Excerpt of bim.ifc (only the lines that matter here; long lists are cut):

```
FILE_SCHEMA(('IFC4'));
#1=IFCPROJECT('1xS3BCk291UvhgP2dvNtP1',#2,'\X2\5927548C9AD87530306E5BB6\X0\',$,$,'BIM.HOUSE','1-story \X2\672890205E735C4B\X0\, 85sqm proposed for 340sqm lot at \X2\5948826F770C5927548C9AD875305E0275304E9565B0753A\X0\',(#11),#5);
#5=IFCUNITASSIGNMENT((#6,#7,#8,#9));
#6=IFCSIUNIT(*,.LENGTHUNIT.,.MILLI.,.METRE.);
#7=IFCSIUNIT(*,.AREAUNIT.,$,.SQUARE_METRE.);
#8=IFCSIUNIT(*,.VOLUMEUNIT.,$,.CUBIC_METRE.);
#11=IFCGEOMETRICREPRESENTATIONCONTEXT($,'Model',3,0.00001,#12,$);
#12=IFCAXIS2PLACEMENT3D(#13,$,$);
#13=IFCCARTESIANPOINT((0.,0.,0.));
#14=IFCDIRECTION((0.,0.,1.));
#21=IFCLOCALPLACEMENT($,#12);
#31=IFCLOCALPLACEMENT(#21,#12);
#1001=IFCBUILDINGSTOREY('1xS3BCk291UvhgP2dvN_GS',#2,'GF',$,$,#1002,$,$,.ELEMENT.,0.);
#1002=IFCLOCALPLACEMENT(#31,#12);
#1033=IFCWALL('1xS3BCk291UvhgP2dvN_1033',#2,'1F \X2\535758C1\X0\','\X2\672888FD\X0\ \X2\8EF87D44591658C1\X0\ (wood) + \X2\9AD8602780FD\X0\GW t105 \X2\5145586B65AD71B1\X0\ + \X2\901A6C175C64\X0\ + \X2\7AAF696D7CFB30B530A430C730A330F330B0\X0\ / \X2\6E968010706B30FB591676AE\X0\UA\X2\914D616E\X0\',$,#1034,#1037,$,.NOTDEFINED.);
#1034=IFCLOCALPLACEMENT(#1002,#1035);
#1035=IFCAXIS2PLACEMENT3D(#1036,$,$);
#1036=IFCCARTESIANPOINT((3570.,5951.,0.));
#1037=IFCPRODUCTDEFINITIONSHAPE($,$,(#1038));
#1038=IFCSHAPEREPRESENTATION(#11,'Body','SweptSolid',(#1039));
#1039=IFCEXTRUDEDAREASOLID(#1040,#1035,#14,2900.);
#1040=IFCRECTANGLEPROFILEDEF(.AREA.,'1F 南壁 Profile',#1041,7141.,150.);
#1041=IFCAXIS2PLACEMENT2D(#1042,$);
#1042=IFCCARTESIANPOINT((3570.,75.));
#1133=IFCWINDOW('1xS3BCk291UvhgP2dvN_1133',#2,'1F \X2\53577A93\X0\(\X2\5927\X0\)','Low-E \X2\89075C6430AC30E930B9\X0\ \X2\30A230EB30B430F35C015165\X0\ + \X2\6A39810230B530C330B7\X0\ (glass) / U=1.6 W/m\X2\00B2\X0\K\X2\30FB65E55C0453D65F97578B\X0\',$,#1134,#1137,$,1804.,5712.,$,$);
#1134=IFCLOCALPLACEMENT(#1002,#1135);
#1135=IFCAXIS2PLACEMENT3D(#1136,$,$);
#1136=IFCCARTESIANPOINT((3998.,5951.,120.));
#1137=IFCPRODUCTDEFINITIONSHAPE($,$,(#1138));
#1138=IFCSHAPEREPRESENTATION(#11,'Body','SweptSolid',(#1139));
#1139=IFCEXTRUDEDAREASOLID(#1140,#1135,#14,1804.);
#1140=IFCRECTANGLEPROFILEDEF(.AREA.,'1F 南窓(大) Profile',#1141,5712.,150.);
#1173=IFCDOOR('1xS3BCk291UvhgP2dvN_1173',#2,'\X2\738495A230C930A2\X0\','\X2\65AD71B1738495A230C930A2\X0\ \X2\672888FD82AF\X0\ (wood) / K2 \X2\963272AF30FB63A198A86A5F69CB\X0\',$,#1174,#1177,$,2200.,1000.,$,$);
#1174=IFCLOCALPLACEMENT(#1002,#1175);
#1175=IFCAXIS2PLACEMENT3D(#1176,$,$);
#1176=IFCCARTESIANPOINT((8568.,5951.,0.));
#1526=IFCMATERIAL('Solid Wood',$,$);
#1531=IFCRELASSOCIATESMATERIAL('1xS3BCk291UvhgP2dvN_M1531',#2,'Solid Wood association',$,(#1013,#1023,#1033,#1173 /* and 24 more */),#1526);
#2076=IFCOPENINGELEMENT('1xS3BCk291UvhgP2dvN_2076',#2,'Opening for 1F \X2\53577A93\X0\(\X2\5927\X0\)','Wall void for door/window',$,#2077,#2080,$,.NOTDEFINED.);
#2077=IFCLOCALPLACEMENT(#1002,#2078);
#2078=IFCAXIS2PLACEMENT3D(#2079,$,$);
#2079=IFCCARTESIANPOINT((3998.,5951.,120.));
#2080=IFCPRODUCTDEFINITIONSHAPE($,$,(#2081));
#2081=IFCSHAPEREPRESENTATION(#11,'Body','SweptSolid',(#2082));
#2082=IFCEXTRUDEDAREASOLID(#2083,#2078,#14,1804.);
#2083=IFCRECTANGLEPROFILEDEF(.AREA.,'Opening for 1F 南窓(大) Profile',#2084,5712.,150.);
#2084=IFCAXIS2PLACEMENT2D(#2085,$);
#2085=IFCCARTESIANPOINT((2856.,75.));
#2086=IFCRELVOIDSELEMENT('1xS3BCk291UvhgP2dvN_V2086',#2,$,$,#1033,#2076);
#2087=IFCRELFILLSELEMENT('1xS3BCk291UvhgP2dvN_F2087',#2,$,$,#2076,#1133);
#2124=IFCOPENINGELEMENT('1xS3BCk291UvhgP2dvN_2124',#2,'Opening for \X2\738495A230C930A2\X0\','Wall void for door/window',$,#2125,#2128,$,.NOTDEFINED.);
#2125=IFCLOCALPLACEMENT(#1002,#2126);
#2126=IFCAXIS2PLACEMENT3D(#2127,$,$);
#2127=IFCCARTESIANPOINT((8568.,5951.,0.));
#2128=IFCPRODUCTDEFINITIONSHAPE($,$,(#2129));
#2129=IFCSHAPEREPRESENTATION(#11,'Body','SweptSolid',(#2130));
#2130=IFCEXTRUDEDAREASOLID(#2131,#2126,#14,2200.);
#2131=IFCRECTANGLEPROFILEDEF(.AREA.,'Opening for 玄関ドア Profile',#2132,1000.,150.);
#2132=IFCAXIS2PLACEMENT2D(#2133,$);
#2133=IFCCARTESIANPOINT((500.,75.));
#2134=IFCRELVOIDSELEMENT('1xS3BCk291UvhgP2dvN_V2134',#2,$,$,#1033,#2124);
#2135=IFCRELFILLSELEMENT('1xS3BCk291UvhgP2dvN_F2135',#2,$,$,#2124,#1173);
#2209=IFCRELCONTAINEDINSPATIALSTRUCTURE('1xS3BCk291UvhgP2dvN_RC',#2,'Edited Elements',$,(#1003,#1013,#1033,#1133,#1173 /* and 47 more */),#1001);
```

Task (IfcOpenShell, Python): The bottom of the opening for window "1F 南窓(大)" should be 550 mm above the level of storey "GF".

```python
import numpy as np
import ifcopenshell
import ifcopenshell.api.geometry
import ifcopenshell.geom
import ifcopenshell.util.element
import ifcopenshell.util.placement
import ifcopenshell.util.shape
import ifcopenshell.util.unit

model = ifcopenshell.open("bim.ifc")
unit_scale = ifcopenshell.util.unit.calculate_unit_scale(model)

window = model.by_guid("1xS3BCk291UvhgP2dvN_1133")
opening = window.FillsVoids[0].RelatingOpeningElement
storey = ifcopenshell.util.element.get_container(window, ifc_class="IfcBuildingStorey")
level = ifcopenshell.util.placement.get_local_placement(storey.ObjectPlacement)[2, 3]

# The opening's origin need not be at the sill, so measure its lowest point.
shape = ifcopenshell.geom.create_shape(ifcopenshell.geom.settings(), opening)
bottom = ifcopenshell.util.shape.get_shape_bottom_elevation(shape, shape.geometry) / unit_scale
dz = level + 0.55 / unit_scale - bottom

shift = np.array([0.0, 0.0, dz])
# The window is not placed relative to its opening, so move both.
for product in (opening, window):
    matrix = ifcopenshell.util.placement.get_local_placement(product.ObjectPlacement)
    matrix[:3, 3] += shift
    ifcopenshell.api.geometry.edit_object_placement(model, product=product, matrix=matrix, is_si=False)

print(f"moved by {dz * unit_scale:+.3f} m")

model.write("bim_v2.ifc")
```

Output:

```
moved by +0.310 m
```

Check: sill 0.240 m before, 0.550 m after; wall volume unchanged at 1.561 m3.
